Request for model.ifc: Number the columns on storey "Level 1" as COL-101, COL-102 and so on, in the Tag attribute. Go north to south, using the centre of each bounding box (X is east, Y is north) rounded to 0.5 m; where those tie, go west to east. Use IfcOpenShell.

First a look at what the model holds.

```python
import ifcopenshell
import ifcopenshell.util.element
import ifcopenshell.util.placement

model = ifcopenshell.open("model.ifc")
print(model.schema)
storey = next(s for s in model.by_type("IfcBuildingStorey") if s.Name == "Level 1")
columns = [e for e in ifcopenshell.util.element.get_decomposition(storey) if e.is_a("IfcColumn")]
for e in sorted(columns, key=lambda e: e.id()):
    origin = ifcopenshell.util.placement.get_local_placement(e.ObjectPlacement)[:3, 3]
    print(e.id(), e.Tag, e.Name, origin.round(2) + 0.0, sep=" | ")
```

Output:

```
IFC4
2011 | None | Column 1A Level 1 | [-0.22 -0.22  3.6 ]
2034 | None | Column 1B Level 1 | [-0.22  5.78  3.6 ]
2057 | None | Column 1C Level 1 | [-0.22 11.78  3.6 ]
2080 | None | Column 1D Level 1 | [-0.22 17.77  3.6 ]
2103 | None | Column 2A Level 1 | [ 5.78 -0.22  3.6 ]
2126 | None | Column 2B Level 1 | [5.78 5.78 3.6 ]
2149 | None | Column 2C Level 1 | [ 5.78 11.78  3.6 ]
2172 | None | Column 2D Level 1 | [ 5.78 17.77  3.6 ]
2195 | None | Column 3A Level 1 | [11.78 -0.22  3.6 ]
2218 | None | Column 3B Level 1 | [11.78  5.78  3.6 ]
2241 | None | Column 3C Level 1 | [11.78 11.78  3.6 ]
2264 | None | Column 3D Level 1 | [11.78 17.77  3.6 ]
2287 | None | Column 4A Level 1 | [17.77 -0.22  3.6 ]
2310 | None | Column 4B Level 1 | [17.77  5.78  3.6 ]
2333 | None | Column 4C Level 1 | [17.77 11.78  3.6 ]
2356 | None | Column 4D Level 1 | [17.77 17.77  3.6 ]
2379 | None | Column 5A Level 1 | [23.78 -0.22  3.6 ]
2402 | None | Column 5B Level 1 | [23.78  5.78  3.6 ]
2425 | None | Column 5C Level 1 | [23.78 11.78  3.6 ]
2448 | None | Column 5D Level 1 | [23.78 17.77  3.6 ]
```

```python
import ifcopenshell
import ifcopenshell.geom
import ifcopenshell.util.element
import ifcopenshell.util.shape

model = ifcopenshell.open("model.ifc")
settings = ifcopenshell.geom.settings()
settings.set("use-world-coords", True)


def centre(element):
    shape = ifcopenshell.geom.create_shape(settings, element)
    return ifcopenshell.util.shape.get_bbox_centroid(shape.geometry)


storey = next(s for s in model.by_type("IfcBuildingStorey") if s.Name == "Level 1")
columns = [e for e in ifcopenshell.util.element.get_decomposition(storey) if e.is_a("IfcColumn")]

# Insertion points can sit at a corner or the storey origin, so sort by the geometry (in metres).
centres = {e: centre(e) for e in columns}
columns.sort(key=lambda e: (-round(centres[e][1] / 0.5), centres[e][0]))

for i, e in enumerate(columns, start=1):
    number = f"COL-1{i:02d}"
    e.Tag = number
    print(e.id(), number)

model.write("model_v2.ifc")
```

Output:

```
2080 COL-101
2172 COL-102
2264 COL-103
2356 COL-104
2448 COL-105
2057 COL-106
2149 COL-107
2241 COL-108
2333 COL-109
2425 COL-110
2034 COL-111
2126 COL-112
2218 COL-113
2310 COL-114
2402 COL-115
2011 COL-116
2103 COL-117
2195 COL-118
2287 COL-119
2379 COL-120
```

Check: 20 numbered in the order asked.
